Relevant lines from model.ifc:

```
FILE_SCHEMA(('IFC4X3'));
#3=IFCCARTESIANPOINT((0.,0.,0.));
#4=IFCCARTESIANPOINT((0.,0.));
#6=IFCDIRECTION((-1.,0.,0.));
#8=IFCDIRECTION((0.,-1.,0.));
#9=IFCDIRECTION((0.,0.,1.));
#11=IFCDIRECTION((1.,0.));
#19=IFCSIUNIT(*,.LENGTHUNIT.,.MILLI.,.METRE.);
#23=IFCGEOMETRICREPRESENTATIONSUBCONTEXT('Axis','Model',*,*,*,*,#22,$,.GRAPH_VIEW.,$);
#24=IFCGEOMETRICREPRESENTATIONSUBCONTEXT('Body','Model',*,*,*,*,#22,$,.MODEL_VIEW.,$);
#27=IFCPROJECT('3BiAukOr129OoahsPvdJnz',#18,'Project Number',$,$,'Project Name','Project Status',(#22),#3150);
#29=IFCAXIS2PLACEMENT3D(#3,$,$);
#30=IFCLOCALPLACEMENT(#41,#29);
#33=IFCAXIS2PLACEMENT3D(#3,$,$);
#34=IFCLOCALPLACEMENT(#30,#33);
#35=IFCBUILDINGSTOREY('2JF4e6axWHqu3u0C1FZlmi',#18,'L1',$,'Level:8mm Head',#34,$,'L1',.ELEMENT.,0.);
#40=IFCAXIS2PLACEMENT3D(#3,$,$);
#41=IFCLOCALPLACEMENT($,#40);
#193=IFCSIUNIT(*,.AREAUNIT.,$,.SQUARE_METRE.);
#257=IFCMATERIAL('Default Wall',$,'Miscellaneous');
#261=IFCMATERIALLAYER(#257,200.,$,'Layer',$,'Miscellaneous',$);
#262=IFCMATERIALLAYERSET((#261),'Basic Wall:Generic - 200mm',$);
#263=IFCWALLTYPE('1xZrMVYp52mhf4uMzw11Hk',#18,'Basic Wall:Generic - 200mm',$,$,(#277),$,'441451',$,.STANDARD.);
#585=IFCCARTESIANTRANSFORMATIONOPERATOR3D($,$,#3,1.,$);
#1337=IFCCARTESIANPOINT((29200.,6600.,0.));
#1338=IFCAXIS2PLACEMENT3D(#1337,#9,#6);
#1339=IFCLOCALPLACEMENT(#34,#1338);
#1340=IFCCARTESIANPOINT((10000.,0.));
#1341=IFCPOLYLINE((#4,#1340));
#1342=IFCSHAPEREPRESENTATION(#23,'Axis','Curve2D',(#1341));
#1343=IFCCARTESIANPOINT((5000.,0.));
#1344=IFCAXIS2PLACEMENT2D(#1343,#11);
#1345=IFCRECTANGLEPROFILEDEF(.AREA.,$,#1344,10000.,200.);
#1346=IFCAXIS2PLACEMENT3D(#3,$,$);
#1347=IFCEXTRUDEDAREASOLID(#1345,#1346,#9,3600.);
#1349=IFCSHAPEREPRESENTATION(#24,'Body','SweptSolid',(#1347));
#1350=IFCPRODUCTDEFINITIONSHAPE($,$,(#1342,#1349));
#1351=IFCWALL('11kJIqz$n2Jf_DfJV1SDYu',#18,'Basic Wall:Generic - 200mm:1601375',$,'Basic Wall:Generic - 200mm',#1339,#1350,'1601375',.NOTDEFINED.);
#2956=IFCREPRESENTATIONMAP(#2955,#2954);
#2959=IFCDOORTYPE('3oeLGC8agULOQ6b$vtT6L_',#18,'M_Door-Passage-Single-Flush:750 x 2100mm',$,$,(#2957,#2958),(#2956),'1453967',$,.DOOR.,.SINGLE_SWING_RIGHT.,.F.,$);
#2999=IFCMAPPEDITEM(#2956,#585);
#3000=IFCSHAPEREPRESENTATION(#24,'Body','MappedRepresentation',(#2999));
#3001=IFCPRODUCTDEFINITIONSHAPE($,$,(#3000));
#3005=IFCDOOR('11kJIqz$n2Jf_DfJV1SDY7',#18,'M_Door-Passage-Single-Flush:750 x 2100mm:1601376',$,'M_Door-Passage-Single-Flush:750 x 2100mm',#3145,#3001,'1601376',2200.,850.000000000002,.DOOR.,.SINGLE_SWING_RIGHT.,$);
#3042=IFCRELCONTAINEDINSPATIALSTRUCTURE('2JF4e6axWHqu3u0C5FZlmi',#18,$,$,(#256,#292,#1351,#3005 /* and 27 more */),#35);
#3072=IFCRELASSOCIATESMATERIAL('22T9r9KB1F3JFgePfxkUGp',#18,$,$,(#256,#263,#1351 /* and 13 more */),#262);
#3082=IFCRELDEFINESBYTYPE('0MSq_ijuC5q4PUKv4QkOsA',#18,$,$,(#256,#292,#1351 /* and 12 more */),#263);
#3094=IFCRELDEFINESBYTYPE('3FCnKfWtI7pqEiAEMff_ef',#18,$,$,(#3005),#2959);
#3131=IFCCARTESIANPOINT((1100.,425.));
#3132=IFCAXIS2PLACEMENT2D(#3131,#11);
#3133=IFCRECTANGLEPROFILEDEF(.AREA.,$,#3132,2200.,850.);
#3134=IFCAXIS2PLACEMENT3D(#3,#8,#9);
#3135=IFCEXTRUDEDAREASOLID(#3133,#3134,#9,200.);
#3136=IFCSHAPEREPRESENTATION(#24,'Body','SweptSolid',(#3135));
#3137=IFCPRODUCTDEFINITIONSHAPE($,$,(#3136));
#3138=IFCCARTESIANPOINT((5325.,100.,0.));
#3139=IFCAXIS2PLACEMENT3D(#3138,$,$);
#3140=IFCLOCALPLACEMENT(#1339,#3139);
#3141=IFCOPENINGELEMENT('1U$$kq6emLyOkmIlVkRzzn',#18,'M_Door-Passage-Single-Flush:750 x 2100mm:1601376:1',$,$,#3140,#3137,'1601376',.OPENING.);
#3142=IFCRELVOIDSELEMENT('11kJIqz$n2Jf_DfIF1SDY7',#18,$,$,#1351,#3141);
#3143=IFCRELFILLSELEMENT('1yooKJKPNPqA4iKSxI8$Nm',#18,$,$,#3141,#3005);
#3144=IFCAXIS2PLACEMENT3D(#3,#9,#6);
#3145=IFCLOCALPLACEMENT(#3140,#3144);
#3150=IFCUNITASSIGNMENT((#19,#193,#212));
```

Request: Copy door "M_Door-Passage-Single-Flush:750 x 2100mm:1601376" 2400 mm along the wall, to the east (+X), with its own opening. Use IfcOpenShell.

```python
import ifcopenshell
import ifcopenshell.api.feature
import ifcopenshell.api.geometry
import ifcopenshell.api.root
import ifcopenshell.geom
import ifcopenshell.util.element
import ifcopenshell.util.placement
import ifcopenshell.util.shape

model = ifcopenshell.open("model.ifc")
settings = ifcopenshell.geom.settings()


def volume(element):
    """Net volume in cubic metres, openings subtracted."""
    shape = ifcopenshell.geom.create_shape(settings, element)
    return ifcopenshell.util.shape.get_volume(shape.geometry)


def reuse_history(source, copy):
    """copy_class also copies each property set's owner history, people and application; keep the originals."""
    for rel in copy.IsDefinedBy:
        if rel.is_a("IfcRelDefinesByProperties") and (history := rel.RelatingPropertyDefinition.OwnerHistory):
            rel.RelatingPropertyDefinition.OwnerHistory = source.OwnerHistory
            ifcopenshell.util.element.remove_deep2(model, history)


door = model.by_id(3005)
opening = door.FillsVoids[0].RelatingOpeningElement
wall = opening.VoidsElements[0].RelatingBuildingElement
before = volume(wall)
shift = ifcopenshell.util.placement.get_local_placement(wall.ObjectPlacement)[:3, 0] * -2400.0

# copy_class copies the void relationship, type, container and properties, but no geometry.
new_opening = ifcopenshell.api.root.copy_class(model, product=opening)
new_opening.Representation = ifcopenshell.util.element.copy_deep(
    model, opening.Representation, exclude=["IfcGeometricRepresentationContext", "IfcRepresentationMap"]
)
new_opening.Name = "M_Door-Passage-Single-Flush:750 x 2100mm"
new_opening.Tag = None
new_door = ifcopenshell.api.root.copy_class(model, product=door)
new_door.Representation = ifcopenshell.util.element.copy_deep(
    model, door.Representation, exclude=["IfcGeometricRepresentationContext", "IfcRepresentationMap"]
)
new_door.Name = "M_Door-Passage-Single-Flush:750 x 2100mm"
new_door.Tag = None
reuse_history(door, new_door)
ifcopenshell.api.feature.add_filling(model, opening=new_opening, element=new_door)

for old, new in ((opening, new_opening), (door, new_door)):
    matrix = ifcopenshell.util.placement.get_local_placement(old.ObjectPlacement)
    matrix[:3, 3] += shift
    ifcopenshell.api.geometry.edit_object_placement(model, product=new, matrix=matrix, is_si=False)

after = volume(wall)

print(f"wall volume {before:.3f} -> {after:.3f} m3")

model.write("model-out.ifc")
```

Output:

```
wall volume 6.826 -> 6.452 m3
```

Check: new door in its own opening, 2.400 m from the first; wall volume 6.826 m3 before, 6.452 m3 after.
